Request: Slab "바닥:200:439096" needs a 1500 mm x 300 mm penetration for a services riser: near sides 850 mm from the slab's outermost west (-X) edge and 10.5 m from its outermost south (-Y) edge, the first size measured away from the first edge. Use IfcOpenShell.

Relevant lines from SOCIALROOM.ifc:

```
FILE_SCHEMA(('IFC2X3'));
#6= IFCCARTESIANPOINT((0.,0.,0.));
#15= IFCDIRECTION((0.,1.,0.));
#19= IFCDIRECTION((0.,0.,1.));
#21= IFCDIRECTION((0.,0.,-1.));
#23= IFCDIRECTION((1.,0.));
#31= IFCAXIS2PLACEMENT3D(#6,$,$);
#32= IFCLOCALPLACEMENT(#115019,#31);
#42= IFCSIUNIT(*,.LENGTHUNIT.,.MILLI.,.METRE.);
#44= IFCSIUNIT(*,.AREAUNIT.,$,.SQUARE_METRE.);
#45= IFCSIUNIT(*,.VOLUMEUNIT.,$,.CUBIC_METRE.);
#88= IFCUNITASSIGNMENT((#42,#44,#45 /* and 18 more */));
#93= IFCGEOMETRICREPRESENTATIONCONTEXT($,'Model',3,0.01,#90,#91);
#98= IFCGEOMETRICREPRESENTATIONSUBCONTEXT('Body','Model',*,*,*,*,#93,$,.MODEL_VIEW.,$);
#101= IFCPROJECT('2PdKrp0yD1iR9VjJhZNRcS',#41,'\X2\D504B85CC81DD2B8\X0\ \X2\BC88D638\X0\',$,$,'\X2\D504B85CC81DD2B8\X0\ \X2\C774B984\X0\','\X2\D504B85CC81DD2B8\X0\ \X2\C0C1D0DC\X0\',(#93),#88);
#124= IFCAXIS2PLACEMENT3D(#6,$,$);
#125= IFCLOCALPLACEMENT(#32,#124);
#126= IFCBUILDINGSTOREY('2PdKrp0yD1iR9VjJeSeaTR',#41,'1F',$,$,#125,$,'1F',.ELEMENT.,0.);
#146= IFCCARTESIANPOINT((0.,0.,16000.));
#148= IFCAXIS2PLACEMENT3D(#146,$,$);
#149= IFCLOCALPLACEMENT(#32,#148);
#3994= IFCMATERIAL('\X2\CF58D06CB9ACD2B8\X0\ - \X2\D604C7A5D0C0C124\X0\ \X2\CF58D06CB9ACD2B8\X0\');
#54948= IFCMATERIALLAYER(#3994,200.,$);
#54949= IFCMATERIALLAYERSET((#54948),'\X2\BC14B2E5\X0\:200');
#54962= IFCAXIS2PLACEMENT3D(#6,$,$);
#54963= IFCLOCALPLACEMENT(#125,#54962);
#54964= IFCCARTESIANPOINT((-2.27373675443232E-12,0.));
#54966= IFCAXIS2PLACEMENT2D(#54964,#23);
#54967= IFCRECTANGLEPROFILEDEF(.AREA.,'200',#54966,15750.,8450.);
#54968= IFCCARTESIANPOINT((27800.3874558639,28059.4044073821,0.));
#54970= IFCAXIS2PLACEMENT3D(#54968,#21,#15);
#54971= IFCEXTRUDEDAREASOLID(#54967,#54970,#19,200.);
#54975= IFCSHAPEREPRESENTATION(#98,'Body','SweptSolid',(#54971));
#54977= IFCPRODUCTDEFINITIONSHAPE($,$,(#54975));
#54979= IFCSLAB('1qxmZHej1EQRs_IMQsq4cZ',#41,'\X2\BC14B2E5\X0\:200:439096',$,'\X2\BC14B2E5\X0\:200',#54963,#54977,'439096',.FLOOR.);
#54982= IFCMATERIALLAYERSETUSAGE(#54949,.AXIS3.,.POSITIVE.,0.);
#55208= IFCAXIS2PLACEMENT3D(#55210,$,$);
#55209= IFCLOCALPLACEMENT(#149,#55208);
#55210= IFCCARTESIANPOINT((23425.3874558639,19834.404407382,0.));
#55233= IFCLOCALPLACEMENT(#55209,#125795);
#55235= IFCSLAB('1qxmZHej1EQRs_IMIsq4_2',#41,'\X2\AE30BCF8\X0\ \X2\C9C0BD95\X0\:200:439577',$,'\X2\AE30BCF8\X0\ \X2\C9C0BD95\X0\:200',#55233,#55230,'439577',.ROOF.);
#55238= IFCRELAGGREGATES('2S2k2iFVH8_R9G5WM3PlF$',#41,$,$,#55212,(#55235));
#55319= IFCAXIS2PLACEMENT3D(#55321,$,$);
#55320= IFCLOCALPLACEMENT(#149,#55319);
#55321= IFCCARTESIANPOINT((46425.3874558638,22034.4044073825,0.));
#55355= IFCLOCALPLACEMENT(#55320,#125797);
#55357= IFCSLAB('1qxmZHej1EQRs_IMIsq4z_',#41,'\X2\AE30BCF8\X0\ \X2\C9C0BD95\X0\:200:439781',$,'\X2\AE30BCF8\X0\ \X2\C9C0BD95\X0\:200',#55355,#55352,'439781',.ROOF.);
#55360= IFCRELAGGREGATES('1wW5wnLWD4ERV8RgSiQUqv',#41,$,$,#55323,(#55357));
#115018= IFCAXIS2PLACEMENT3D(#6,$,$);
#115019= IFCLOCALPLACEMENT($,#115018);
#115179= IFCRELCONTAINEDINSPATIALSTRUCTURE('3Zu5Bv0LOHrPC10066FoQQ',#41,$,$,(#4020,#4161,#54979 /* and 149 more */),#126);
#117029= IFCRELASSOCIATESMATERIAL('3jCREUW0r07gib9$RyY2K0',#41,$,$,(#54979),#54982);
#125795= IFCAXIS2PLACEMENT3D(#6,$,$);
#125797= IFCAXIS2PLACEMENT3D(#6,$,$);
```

```python
import numpy as np
import ifcopenshell
import ifcopenshell.api.feature
import ifcopenshell.api.geometry
import ifcopenshell.api.root
import ifcopenshell.geom
import ifcopenshell.util.placement
import ifcopenshell.util.representation
import ifcopenshell.util.shape
import ifcopenshell.util.unit

model = ifcopenshell.open("SOCIALROOM.ifc")
unit_scale = ifcopenshell.util.unit.calculate_unit_scale(model)
settings = ifcopenshell.geom.settings()


def volume(element):
    """Net volume in cubic metres, openings subtracted."""
    shape = ifcopenshell.geom.create_shape(settings, element)
    return ifcopenshell.util.shape.get_volume(shape.geometry)


slab = model.by_guid("1qxmZHej1EQRs_IMQsq4cZ")
before = volume(slab)

# Extent in the slab's own axes, in metres. The edges named are its -X and -Y sides.
slab_shape = ifcopenshell.geom.create_shape(settings, slab)
vertices = ifcopenshell.util.shape.get_vertices(slab_shape.geometry)
x_min, y_min, bottom = vertices.min(axis=0)
top = vertices[:, 2].max()

opening = ifcopenshell.api.root.create_entity(model, ifc_class="IfcOpeningElement", name="Services riser opening")
context = ifcopenshell.util.representation.get_context(model, "Model", "Body", "MODEL_VIEW")
width, depth = 1.5, 0.3
outline = [(0.0, 0.0), (width, 0.0), (width, depth), (0.0, depth), (0.0, 0.0)]
# Overshoot both faces by 50 mm so the cut is clean.
shape = ifcopenshell.api.geometry.add_slab_representation(
    model, context=context, depth=top - bottom + 0.1, polyline=outline
)
ifcopenshell.api.geometry.assign_representation(model, product=opening, representation=shape)

matrix = ifcopenshell.util.placement.get_local_placement(slab.ObjectPlacement)
matrix[:, 3] = matrix @ np.append(np.array([x_min + 0.85, y_min + 10.5, bottom - 0.05]) / unit_scale, 1.0)
ifcopenshell.api.geometry.edit_object_placement(model, product=opening, matrix=matrix, is_si=False)
ifcopenshell.api.feature.add_feature(model, feature=opening, element=slab)

after = volume(slab)

print(f"slab volume {before:.3f} -> {after:.3f} m3")

model.write("SOCIALROOM_edited.ifc")
```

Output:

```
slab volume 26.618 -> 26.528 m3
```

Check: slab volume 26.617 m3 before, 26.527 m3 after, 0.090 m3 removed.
